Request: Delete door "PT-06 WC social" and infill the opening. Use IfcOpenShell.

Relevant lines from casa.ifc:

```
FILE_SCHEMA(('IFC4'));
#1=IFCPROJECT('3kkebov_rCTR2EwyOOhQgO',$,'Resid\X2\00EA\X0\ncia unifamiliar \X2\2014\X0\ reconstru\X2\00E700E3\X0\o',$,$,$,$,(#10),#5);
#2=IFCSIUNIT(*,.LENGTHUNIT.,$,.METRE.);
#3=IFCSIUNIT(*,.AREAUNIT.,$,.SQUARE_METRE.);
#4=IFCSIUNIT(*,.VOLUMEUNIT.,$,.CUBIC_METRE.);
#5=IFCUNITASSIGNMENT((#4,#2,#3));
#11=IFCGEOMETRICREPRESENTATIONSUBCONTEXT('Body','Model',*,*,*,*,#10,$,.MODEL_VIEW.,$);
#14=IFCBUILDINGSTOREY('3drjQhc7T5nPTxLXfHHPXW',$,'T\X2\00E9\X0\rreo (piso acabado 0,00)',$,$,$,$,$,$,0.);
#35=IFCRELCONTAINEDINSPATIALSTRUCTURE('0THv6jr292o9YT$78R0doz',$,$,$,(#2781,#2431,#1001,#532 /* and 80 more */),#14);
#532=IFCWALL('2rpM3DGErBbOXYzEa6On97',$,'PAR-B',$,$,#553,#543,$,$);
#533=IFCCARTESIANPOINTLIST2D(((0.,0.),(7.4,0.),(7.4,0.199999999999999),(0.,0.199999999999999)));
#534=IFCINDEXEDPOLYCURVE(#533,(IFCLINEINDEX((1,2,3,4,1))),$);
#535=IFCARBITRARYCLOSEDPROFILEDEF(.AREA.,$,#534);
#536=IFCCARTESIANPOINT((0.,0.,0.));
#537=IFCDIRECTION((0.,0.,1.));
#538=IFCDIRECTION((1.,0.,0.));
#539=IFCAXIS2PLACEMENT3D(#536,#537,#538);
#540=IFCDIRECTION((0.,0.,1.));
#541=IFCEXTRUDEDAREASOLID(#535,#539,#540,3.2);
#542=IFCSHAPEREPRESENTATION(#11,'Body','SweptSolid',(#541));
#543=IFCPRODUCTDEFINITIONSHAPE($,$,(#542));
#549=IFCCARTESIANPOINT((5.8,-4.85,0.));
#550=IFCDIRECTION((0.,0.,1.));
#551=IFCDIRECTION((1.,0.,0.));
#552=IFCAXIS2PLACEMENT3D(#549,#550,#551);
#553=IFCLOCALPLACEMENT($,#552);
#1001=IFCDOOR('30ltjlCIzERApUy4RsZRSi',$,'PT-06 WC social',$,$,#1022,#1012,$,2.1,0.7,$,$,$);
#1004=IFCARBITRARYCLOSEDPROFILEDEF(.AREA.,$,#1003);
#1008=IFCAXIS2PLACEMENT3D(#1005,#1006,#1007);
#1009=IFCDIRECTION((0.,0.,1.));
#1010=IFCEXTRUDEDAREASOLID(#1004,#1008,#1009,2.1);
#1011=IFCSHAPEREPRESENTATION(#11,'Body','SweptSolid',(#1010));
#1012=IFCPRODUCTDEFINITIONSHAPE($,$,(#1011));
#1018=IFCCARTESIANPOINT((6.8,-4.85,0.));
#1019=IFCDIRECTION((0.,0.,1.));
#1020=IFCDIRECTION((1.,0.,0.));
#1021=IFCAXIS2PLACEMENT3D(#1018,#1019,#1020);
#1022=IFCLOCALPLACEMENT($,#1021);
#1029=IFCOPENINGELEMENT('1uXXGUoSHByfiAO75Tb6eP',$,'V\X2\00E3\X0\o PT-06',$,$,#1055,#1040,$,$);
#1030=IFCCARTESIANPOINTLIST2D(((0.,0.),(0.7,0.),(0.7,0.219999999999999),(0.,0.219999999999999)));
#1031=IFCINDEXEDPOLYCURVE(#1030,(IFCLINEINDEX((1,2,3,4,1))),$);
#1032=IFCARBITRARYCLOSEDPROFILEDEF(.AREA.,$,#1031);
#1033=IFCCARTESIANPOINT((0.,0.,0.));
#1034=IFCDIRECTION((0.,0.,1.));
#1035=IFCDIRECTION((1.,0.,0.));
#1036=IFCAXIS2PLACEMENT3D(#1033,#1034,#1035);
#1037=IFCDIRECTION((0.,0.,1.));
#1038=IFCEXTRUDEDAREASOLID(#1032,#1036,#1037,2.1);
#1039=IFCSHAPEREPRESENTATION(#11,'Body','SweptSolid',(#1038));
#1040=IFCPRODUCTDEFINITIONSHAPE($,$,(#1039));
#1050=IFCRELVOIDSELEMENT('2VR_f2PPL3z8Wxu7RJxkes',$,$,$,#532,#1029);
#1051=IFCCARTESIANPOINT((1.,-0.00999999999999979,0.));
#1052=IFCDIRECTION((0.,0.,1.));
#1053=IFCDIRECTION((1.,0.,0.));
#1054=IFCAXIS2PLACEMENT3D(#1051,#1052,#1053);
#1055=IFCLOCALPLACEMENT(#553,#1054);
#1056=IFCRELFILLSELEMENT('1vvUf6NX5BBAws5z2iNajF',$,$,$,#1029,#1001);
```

```python
import ifcopenshell
import ifcopenshell.api.feature
import ifcopenshell.api.root
import ifcopenshell.geom
import ifcopenshell.util.shape

model = ifcopenshell.open("casa.ifc")
settings = ifcopenshell.geom.settings()


def volume(element):
    """Net volume in cubic metres, openings subtracted."""
    shape = ifcopenshell.geom.create_shape(settings, element)
    return ifcopenshell.util.shape.get_volume(shape.geometry)


door = model.by_guid("30ltjlCIzERApUy4RsZRSi")
opening = door.FillsVoids[0].RelatingOpeningElement
wall = opening.VoidsElements[0].RelatingBuildingElement
before = volume(wall)

ifcopenshell.api.root.remove_product(model, product=door)
ifcopenshell.api.feature.remove_feature(model, feature=opening)

after = volume(wall)

print(f"wall volume {before:.3f} -> {after:.3f} m3")

model.write("casa-out.ifc")
```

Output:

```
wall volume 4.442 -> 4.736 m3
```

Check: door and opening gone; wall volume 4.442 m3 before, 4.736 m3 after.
